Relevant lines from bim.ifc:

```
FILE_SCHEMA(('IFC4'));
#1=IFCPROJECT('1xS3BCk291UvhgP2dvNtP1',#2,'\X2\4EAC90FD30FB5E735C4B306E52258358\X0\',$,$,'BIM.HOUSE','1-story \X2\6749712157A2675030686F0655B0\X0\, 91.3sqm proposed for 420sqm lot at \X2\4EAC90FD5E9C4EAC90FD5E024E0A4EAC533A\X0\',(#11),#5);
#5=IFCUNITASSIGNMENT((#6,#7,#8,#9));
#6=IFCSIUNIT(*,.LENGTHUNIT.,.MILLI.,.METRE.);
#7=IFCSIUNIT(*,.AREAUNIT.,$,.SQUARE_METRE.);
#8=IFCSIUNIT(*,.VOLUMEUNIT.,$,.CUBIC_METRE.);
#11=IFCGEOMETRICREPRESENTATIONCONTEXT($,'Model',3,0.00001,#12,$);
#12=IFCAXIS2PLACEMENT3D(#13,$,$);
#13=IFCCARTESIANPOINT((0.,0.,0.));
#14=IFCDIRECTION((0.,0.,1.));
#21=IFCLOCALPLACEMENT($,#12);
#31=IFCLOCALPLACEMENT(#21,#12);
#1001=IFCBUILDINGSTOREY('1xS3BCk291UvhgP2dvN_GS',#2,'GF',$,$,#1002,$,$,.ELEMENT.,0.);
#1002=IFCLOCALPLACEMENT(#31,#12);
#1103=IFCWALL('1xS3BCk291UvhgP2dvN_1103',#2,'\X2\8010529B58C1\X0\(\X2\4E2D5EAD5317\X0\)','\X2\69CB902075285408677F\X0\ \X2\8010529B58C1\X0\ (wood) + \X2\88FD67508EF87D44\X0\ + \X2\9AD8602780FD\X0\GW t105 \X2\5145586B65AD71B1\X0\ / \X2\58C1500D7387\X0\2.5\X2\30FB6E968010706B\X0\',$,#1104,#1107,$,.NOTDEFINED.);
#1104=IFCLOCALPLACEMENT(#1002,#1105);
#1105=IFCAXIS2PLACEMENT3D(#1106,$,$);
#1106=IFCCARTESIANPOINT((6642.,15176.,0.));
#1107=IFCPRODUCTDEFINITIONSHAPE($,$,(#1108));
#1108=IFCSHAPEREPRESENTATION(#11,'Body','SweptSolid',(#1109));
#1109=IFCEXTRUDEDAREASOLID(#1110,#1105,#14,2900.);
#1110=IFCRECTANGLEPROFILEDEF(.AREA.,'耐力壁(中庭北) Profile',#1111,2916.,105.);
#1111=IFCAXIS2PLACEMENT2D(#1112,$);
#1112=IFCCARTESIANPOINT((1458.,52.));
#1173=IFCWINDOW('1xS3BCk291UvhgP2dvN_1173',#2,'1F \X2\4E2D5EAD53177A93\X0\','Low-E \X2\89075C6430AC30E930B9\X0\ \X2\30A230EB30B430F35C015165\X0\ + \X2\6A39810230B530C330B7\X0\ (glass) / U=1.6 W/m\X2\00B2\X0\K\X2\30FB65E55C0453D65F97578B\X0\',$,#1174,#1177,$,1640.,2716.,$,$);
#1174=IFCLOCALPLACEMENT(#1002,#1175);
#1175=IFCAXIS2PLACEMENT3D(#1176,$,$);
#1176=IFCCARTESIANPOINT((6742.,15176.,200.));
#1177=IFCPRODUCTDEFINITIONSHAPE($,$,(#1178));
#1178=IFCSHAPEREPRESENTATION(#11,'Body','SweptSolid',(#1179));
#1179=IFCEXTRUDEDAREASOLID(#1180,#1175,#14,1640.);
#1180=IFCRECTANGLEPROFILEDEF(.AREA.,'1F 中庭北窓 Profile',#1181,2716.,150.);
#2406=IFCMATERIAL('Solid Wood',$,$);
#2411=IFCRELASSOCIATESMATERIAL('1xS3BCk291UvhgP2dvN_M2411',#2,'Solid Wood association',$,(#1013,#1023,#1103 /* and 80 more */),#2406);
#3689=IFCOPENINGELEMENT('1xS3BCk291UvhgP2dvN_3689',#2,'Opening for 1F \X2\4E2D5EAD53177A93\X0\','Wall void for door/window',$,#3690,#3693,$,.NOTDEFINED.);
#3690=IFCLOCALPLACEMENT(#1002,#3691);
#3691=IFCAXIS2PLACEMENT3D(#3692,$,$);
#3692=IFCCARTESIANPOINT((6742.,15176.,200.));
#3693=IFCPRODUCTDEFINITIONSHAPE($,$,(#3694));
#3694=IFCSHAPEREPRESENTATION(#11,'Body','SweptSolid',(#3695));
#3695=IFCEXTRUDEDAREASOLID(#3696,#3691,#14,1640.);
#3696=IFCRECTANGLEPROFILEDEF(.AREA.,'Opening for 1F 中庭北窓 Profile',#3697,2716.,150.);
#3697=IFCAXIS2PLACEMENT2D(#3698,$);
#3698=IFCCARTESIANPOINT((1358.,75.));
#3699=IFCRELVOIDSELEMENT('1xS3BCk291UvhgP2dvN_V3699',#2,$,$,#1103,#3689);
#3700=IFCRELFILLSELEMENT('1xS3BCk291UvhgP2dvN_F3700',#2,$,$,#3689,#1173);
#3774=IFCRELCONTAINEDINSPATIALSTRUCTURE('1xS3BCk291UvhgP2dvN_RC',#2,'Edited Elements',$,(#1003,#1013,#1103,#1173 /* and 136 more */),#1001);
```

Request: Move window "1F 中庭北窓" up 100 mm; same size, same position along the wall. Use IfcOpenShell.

```python
import numpy as np
import ifcopenshell
import ifcopenshell.api.geometry
import ifcopenshell.util.placement
import ifcopenshell.util.unit

model = ifcopenshell.open("bim.ifc")
unit_scale = ifcopenshell.util.unit.calculate_unit_scale(model)

window = model.by_guid("1xS3BCk291UvhgP2dvN_1173")
opening = window.FillsVoids[0].RelatingOpeningElement
dz = 0.1 / unit_scale

shift = np.array([0.0, 0.0, dz])
# The window is not placed relative to its opening, so move both.
for product in (opening, window):
    matrix = ifcopenshell.util.placement.get_local_placement(product.ObjectPlacement)
    matrix[:3, 3] += shift
    ifcopenshell.api.geometry.edit_object_placement(model, product=product, matrix=matrix, is_si=False)

print(f"moved by {dz * unit_scale:+.3f} m")

model.write("bim-out.ifc")
```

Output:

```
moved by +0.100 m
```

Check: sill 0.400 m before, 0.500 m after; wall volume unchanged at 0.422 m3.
